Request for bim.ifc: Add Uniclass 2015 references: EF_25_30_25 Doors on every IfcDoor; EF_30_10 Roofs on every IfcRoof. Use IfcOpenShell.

First a look at what the model holds.

```python
import ifcopenshell

model = ifcopenshell.open("bim.ifc")
print(model.schema)
print("classifications:", [c.Name for c in model.by_type("IfcClassification")])
for ifc_class in ("IfcDoor", "IfcRoof", "IfcStair", "IfcWall", "IfcWindow"):
    print(ifc_class, len(model.by_type(ifc_class)))
```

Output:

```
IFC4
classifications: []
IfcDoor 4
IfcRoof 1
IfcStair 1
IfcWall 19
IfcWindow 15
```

```python
import ifcopenshell
import ifcopenshell.api.classification

model = ifcopenshell.open("bim.ifc")

system = ifcopenshell.api.classification.add_classification(model, classification="Uniclass 2015")

codes = {
    "IfcDoor": ("EF_25_30_25", "Doors"),
    "IfcRoof": ("EF_30_10", "Roofs"),
}
for ifc_class, (code, name) in codes.items():
    products = model.by_type(ifc_class)
    ifcopenshell.api.classification.add_reference(
        model, products=products, classification=system, identification=code, name=name
    )
    print(code, len(products))

model.write("bim_updated.ifc")
```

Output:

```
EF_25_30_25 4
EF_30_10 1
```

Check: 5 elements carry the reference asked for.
